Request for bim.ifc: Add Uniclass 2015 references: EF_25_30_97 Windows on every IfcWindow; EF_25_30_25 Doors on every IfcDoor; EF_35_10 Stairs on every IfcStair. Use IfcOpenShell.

First a look at what the model holds.

```python
import ifcopenshell

model = ifcopenshell.open("bim.ifc")
print(model.schema)
print("classifications:", [c.Name for c in model.by_type("IfcClassification")])
for ifc_class in ("IfcDoor", "IfcRoof", "IfcStair", "IfcWall", "IfcWindow"):
    print(ifc_class, len(model.by_type(ifc_class)))
```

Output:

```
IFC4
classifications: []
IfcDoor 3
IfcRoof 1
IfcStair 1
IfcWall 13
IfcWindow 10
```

```python
import ifcopenshell
import ifcopenshell.api.classification

model = ifcopenshell.open("bim.ifc")

system = ifcopenshell.api.classification.add_classification(model, classification="Uniclass 2015")

codes = {
    "IfcWindow": ("EF_25_30_97", "Windows"),
    "IfcDoor": ("EF_25_30_25", "Doors"),
    "IfcStair": ("EF_35_10", "Stairs"),
}
for ifc_class, (code, name) in codes.items():
    products = model.by_type(ifc_class)
    ifcopenshell.api.classification.add_reference(
        model, products=products, classification=system, identification=code, name=name
    )
    print(code, len(products))

model.write("bim_v2.ifc")
```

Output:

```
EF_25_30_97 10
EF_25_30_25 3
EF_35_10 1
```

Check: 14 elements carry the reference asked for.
